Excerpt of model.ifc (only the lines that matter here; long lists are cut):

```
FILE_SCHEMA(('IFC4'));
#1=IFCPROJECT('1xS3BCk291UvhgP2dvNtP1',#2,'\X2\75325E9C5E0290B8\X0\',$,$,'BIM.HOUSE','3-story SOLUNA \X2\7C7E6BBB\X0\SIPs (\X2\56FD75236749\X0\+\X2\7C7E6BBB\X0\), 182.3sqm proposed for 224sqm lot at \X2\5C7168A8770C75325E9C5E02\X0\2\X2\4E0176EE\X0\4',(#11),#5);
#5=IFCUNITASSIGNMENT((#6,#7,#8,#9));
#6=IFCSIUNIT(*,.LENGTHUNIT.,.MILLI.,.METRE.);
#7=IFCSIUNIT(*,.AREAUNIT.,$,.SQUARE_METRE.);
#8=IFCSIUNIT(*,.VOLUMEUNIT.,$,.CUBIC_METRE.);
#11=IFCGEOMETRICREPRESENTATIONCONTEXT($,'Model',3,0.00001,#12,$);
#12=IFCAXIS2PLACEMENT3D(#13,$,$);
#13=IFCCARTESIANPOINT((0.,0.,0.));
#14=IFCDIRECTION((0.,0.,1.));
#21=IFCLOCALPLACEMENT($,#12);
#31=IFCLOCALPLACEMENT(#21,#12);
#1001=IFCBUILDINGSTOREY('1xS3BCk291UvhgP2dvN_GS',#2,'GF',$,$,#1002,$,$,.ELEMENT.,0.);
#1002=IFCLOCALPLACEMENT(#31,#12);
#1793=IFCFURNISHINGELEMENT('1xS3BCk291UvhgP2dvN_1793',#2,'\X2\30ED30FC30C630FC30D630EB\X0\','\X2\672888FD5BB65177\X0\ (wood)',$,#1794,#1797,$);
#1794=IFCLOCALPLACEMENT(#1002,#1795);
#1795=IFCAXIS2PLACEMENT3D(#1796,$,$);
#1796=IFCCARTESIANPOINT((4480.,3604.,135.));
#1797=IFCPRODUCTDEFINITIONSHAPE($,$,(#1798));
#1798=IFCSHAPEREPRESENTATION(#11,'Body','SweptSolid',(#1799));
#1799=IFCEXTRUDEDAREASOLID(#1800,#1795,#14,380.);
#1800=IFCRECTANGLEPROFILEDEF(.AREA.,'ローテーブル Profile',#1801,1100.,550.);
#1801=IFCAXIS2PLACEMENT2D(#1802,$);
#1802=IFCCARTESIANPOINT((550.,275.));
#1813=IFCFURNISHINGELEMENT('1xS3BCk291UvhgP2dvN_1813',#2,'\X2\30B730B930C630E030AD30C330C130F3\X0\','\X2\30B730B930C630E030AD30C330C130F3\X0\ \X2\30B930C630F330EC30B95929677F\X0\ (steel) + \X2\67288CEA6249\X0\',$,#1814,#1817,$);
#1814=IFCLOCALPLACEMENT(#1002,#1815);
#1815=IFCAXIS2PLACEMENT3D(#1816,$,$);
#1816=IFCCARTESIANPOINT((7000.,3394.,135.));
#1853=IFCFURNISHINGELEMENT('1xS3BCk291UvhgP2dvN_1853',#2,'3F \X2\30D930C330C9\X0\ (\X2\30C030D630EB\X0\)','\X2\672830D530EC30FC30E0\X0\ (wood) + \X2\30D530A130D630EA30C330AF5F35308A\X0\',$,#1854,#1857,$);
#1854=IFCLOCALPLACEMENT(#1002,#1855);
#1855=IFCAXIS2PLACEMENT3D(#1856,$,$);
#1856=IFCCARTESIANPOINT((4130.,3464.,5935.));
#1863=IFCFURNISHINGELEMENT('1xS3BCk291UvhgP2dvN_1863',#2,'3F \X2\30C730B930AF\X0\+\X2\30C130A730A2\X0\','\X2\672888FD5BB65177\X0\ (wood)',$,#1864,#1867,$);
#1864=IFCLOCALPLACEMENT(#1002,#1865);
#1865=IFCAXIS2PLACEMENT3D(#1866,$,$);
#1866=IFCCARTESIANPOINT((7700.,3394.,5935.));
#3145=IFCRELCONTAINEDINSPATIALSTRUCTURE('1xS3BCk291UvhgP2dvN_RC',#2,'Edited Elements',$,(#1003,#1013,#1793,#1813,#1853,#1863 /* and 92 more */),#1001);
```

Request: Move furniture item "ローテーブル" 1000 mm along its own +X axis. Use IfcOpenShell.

```python
import ifcopenshell
import ifcopenshell.api.geometry
import ifcopenshell.util.placement
import ifcopenshell.util.unit

model = ifcopenshell.open("model.ifc")
unit_scale = ifcopenshell.util.unit.calculate_unit_scale(model)

item = model.by_id(1793)
matrix = ifcopenshell.util.placement.get_local_placement(item.ObjectPlacement)
matrix[:3, 3] += matrix[:3, 0] * 1 / unit_scale
ifcopenshell.api.geometry.edit_object_placement(model, product=item, matrix=matrix, is_si=False)

print(ifcopenshell.util.placement.get_local_placement(item.ObjectPlacement).round(3) + 0.0)

model.write("model-out.ifc")
```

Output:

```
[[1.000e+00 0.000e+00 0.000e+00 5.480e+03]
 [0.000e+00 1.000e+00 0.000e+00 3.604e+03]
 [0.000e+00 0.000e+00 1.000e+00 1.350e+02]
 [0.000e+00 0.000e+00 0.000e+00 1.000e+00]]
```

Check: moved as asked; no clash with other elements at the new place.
